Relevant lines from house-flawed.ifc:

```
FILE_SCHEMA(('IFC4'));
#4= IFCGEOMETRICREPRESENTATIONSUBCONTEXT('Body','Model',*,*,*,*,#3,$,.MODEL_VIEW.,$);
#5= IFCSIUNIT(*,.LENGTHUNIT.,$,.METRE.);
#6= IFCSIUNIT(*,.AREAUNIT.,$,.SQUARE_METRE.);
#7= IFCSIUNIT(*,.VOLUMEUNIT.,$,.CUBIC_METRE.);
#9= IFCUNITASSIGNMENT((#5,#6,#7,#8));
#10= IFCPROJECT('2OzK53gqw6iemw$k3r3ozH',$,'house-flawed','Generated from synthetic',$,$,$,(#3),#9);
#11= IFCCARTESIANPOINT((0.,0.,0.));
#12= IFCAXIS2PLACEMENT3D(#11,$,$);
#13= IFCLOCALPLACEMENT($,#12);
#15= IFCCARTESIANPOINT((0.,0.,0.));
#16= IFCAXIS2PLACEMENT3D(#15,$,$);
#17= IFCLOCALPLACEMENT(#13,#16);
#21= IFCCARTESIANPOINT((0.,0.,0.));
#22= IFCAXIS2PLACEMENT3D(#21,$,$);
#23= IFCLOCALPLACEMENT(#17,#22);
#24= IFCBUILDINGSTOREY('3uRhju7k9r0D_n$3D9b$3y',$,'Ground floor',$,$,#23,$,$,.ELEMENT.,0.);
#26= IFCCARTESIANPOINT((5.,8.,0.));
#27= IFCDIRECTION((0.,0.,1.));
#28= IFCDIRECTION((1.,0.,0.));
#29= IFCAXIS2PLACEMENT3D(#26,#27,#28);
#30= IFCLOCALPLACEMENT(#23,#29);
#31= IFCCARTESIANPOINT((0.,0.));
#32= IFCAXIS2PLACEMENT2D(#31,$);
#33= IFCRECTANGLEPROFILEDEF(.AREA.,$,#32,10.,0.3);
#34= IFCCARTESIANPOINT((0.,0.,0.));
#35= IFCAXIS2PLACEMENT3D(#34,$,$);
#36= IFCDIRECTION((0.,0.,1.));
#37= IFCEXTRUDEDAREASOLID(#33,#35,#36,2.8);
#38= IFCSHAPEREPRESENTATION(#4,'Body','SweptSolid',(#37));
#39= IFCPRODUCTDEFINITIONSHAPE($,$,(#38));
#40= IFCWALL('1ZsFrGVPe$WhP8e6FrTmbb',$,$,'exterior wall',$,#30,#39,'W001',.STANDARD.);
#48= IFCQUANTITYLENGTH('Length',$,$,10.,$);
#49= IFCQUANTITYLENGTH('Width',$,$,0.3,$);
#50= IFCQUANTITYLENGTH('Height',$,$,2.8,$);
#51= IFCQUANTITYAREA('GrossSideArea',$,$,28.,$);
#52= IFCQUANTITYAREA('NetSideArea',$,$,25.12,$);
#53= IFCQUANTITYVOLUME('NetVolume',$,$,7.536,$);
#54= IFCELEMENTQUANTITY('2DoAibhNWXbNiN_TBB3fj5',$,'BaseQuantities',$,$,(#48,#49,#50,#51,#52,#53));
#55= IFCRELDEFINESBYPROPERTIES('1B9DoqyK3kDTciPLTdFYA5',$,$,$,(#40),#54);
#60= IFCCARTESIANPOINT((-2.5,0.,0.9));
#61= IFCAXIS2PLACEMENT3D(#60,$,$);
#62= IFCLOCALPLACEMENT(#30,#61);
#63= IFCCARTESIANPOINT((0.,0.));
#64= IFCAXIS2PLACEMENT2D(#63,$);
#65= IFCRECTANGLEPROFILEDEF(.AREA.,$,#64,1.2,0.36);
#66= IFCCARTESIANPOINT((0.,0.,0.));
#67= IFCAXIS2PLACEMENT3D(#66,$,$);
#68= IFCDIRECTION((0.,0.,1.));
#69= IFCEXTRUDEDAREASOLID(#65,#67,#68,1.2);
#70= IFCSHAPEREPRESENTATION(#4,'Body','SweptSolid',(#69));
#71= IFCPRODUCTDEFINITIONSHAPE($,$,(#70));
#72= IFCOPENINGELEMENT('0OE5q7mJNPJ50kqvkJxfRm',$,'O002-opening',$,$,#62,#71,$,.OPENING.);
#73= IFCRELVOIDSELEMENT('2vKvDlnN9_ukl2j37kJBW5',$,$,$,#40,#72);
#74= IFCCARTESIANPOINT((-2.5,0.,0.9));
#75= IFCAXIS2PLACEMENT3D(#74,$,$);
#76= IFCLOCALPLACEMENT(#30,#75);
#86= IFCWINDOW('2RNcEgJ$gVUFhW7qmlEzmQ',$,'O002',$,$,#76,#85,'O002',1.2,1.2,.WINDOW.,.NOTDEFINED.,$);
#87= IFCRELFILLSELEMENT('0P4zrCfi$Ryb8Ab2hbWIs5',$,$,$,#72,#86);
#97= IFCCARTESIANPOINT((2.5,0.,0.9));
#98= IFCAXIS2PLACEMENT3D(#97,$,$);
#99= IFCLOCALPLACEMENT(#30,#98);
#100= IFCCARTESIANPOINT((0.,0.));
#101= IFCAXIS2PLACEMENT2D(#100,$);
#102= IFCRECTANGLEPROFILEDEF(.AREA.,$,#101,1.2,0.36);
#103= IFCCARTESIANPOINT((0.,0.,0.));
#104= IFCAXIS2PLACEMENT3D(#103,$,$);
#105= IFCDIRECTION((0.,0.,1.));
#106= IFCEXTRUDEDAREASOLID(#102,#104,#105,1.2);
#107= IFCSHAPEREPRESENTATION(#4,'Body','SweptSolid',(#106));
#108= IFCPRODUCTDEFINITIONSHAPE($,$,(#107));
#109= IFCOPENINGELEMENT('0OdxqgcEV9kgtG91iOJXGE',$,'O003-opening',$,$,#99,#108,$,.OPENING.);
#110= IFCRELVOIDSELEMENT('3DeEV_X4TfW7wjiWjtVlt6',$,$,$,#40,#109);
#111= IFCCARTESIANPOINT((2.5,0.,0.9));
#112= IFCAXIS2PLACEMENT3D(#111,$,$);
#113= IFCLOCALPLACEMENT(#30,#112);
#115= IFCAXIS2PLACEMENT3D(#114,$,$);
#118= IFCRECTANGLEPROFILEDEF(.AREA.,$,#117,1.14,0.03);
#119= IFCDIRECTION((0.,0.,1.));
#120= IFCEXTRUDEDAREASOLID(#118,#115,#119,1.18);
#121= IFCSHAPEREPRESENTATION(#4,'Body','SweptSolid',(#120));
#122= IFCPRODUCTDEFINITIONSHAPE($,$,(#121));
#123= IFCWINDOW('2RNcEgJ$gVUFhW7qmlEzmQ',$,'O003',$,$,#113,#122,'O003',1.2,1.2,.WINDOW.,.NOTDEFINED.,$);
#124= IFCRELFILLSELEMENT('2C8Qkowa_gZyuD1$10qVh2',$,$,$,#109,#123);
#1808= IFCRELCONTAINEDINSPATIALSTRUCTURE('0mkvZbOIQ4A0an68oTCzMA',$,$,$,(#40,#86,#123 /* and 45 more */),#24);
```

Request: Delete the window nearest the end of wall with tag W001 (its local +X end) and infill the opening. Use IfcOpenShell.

```python
import ifcopenshell
import ifcopenshell.api.feature
import ifcopenshell.api.pset
import ifcopenshell.api.root
import ifcopenshell.geom
import ifcopenshell.util.element
import ifcopenshell.util.shape
import ifcopenshell.util.unit

model = ifcopenshell.open("house-flawed.ifc")
area_scale = ifcopenshell.util.unit.calculate_unit_scale(model, "AREAUNIT")
volume_scale = ifcopenshell.util.unit.calculate_unit_scale(model, "VOLUMEUNIT")
settings = ifcopenshell.geom.settings()


def volume(element):
    """Net volume in cubic metres, openings subtracted."""
    shape = ifcopenshell.geom.create_shape(settings, element)
    return ifcopenshell.util.shape.get_volume(shape.geometry)


window = model.by_id(123)
opening = window.FillsVoids[0].RelatingOpeningElement
wall = opening.VoidsElements[0].RelatingBuildingElement
before = volume(wall)

ifcopenshell.api.root.remove_product(model, product=window)
ifcopenshell.api.feature.remove_feature(model, feature=opening)

after = volume(wall)
thickness = 0.3  # wall thickness in metres

# Update the wall's stored quantities.
qto = model.by_id(ifcopenshell.util.element.get_pset(wall, "BaseQuantities", should_inherit=False)["id"])
ifcopenshell.api.pset.edit_qto(model, qto=qto, properties={
    "NetSideArea": after / thickness / area_scale,
    "NetVolume": after / volume_scale,
})

print(f"wall volume {before:.3f} -> {after:.3f} m3")

model.write("house-flawed_updated.ifc")
```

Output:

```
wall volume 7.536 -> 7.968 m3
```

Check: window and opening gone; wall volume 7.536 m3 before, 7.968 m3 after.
